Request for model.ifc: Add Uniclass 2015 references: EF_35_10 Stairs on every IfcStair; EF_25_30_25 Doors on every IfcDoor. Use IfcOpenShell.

First a look at what the model holds.

```python
import ifcopenshell

model = ifcopenshell.open("model.ifc")
print(model.schema)
print("classifications:", [c.Name for c in model.by_type("IfcClassification")])
for ifc_class in ("IfcDoor", "IfcRoof", "IfcStair", "IfcWall", "IfcWindow"):
    print(ifc_class, len(model.by_type(ifc_class)))
```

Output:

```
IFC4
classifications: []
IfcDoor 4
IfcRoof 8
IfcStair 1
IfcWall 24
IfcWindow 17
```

```python
import ifcopenshell
import ifcopenshell.api.classification

model = ifcopenshell.open("model.ifc")

system = ifcopenshell.api.classification.add_classification(model, classification="Uniclass 2015")

codes = {
    "IfcStair": ("EF_35_10", "Stairs"),
    "IfcDoor": ("EF_25_30_25", "Doors"),
}
for ifc_class, (code, name) in codes.items():
    products = model.by_type(ifc_class)
    ifcopenshell.api.classification.add_reference(
        model, products=products, classification=system, identification=code, name=name
    )
    print(code, len(products))

model.write("model_updated.ifc")
```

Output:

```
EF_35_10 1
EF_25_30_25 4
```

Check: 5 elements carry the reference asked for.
